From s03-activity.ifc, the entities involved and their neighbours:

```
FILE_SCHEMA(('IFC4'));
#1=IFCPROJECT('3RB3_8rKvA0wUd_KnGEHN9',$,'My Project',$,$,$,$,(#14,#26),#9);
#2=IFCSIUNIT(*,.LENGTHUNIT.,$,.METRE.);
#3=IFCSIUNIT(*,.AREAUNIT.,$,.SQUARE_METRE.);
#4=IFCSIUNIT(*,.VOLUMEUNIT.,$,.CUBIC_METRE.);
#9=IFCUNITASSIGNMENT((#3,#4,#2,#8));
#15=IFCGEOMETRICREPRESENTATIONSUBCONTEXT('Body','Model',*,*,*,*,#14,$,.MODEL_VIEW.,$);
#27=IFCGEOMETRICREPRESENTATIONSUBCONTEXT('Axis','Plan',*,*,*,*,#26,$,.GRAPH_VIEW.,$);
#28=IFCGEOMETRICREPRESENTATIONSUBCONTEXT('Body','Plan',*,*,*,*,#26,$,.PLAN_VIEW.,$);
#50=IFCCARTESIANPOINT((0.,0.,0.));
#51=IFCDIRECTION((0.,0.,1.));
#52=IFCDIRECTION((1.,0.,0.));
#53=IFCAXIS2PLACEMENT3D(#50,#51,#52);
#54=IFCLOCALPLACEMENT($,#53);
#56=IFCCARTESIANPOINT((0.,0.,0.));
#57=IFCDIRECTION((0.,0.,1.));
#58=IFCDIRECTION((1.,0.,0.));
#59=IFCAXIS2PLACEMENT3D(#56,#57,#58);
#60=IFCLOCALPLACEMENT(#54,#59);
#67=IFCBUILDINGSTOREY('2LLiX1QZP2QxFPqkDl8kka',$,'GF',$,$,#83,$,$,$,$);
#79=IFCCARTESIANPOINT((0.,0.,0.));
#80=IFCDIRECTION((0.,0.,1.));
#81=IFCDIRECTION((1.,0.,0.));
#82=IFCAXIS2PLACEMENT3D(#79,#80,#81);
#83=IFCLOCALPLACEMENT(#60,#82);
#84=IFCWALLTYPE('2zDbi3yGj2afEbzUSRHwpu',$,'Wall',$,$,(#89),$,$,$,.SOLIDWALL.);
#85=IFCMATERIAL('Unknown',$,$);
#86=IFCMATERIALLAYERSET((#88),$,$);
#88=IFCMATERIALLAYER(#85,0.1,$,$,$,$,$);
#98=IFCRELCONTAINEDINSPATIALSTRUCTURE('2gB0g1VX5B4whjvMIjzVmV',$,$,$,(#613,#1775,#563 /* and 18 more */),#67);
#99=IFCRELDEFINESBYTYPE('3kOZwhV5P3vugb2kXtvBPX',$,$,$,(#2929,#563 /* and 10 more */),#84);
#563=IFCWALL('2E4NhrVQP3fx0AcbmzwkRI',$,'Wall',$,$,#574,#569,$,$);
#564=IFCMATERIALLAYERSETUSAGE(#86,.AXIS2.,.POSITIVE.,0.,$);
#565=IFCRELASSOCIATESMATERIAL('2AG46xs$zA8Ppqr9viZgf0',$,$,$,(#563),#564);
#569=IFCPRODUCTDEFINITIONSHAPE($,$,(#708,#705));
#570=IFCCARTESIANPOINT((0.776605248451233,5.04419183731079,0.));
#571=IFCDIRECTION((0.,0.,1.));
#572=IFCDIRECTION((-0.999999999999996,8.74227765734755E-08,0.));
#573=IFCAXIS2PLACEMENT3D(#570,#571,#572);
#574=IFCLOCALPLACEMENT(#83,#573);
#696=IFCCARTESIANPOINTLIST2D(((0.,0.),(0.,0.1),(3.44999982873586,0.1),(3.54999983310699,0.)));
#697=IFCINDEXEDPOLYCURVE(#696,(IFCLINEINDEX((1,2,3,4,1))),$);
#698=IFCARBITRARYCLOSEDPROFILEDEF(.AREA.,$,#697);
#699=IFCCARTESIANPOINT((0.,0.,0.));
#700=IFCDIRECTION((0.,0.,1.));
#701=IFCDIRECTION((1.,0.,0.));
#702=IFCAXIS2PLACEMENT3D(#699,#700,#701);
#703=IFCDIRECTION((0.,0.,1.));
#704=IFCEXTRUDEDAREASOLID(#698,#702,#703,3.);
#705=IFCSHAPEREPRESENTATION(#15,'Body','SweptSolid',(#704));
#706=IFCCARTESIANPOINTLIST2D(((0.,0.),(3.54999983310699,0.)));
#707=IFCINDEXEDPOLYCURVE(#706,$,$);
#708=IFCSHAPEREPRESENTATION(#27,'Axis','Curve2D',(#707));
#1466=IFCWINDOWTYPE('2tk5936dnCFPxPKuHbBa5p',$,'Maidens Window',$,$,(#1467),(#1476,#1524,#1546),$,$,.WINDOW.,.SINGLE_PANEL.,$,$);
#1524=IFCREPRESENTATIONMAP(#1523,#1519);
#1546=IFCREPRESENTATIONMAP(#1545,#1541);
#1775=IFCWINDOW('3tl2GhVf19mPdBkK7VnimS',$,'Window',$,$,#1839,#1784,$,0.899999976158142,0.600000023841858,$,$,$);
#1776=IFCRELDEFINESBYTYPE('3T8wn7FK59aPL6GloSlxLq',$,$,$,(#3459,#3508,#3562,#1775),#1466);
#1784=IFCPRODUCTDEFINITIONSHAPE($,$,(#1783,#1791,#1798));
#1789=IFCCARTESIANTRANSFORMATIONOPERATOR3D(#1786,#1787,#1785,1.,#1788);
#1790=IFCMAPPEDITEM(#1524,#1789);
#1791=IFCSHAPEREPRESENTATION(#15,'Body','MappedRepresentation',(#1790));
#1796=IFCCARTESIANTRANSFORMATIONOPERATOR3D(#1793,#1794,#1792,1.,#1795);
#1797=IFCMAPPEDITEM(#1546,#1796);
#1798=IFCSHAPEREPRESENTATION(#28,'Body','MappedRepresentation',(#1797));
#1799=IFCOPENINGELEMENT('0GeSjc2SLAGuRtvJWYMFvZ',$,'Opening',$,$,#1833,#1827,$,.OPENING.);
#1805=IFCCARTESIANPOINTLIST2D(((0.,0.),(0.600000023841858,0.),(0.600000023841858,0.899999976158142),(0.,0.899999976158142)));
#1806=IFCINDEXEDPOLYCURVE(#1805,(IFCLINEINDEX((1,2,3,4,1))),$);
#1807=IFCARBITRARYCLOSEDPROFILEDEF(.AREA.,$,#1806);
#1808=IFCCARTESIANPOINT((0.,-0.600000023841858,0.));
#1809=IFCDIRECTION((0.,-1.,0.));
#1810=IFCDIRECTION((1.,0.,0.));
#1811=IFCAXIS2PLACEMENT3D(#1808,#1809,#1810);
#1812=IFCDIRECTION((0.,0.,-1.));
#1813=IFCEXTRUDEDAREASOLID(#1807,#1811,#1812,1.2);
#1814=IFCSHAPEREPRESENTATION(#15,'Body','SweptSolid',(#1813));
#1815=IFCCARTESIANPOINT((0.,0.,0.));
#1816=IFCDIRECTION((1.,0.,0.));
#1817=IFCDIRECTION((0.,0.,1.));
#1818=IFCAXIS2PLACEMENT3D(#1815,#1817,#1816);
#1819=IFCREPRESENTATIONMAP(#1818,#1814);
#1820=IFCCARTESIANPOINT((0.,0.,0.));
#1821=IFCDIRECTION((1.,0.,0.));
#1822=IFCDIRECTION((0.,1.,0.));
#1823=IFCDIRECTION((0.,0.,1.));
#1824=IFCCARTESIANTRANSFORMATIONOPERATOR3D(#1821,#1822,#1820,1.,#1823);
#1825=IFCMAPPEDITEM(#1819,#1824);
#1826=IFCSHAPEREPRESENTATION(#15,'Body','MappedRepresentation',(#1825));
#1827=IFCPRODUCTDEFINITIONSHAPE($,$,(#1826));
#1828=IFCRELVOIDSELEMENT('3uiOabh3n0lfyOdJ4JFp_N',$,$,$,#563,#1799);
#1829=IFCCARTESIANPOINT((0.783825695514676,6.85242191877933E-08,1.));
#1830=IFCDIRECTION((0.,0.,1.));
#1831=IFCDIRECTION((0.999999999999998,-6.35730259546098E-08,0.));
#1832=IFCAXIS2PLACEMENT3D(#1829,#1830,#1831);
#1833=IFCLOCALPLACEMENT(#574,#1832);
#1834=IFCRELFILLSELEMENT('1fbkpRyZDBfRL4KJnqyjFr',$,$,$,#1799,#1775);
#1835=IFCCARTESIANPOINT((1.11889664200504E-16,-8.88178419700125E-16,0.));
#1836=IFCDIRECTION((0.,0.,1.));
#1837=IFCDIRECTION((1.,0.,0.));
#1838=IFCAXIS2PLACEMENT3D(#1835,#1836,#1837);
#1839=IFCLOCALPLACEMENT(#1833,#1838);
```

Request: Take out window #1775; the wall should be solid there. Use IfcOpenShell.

```python
import ifcopenshell
import ifcopenshell.api.feature
import ifcopenshell.api.root
import ifcopenshell.geom
import ifcopenshell.util.shape

model = ifcopenshell.open("s03-activity.ifc")
settings = ifcopenshell.geom.settings()


def volume(element):
    """Net volume in cubic metres, openings subtracted."""
    shape = ifcopenshell.geom.create_shape(settings, element)
    return ifcopenshell.util.shape.get_volume(shape.geometry)


window = model.by_guid("3tl2GhVf19mPdBkK7VnimS")
opening = window.FillsVoids[0].RelatingOpeningElement
wall = opening.VoidsElements[0].RelatingBuildingElement
before = volume(wall)

ifcopenshell.api.root.remove_product(model, product=window)
ifcopenshell.api.feature.remove_feature(model, feature=opening)

after = volume(wall)

print(f"wall volume {before:.3f} -> {after:.3f} m3")

model.write("s03-activity_edited.ifc")
```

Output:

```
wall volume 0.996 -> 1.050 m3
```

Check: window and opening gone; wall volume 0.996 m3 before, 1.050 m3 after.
